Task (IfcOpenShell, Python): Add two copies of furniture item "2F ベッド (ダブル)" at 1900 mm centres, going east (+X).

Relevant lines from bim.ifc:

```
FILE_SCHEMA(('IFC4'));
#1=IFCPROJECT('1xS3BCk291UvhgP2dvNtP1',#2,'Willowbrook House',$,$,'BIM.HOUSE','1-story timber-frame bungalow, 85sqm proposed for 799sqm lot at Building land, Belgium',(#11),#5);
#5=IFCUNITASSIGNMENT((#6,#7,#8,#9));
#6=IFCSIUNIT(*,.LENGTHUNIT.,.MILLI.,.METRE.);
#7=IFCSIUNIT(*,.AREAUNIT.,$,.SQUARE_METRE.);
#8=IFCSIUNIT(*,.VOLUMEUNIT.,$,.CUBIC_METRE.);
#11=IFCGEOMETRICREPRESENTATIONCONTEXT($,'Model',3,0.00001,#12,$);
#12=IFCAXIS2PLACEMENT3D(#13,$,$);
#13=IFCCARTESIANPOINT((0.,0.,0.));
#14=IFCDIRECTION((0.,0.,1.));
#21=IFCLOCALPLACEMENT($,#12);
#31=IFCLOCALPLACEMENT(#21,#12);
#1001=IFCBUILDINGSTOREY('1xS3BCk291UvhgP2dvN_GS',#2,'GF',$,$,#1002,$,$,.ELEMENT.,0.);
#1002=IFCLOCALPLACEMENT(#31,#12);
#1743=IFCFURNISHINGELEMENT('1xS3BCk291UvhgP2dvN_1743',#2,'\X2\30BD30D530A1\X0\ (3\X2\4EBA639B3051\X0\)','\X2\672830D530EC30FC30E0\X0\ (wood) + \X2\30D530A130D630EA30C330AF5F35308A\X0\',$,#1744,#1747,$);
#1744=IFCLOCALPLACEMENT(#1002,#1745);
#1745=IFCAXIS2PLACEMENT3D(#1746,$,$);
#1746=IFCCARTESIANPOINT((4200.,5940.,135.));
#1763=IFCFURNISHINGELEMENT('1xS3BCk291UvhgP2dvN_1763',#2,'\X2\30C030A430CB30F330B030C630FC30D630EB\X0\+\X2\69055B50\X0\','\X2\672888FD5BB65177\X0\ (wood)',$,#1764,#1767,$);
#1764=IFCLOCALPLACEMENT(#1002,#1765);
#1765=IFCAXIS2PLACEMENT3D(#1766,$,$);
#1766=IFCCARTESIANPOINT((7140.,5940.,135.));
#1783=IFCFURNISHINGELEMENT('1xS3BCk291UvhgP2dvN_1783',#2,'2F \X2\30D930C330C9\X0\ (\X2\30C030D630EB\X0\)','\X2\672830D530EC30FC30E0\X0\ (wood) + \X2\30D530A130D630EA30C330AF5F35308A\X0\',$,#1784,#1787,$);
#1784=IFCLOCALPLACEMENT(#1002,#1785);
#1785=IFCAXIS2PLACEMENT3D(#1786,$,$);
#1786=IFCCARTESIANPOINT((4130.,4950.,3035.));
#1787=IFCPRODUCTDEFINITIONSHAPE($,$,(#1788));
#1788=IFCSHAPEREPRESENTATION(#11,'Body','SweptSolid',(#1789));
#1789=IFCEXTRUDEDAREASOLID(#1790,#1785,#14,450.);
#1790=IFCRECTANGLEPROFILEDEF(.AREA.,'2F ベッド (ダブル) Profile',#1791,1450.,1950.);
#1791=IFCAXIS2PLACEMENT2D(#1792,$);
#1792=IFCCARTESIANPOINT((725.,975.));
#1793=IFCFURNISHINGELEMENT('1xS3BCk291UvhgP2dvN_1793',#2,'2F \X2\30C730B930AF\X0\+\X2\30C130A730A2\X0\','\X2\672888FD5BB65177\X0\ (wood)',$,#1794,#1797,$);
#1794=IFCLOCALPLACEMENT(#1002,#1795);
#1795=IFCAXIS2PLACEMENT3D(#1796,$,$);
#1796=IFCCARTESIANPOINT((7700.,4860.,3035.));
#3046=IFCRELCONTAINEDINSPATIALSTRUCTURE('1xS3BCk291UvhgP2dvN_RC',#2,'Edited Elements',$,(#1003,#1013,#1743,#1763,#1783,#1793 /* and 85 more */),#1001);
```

```python
import numpy as np
import ifcopenshell
import ifcopenshell.api.geometry
import ifcopenshell.api.root
import ifcopenshell.util.element
import ifcopenshell.util.placement
import ifcopenshell.util.unit

model = ifcopenshell.open("bim.ifc")
unit_scale = ifcopenshell.util.unit.calculate_unit_scale(model)


def reuse_history(source, copy):
    """copy_class also copies each property set's owner history, people and application; keep the originals."""
    for rel in copy.IsDefinedBy:
        if rel.is_a("IfcRelDefinesByProperties") and (history := rel.RelatingPropertyDefinition.OwnerHistory):
            rel.RelatingPropertyDefinition.OwnerHistory = source.OwnerHistory
            ifcopenshell.util.element.remove_deep2(model, history)


source = model.by_id(1783)
base = ifcopenshell.util.placement.get_local_placement(source.ObjectPlacement)
step = np.array([1.0, 0.0, 0.0]) * 1.9 / unit_scale

for i in range(1, 3):
    copy = ifcopenshell.api.root.copy_class(model, product=source)
    copy.Representation = ifcopenshell.util.element.copy_deep(
        model, source.Representation, exclude=["IfcGeometricRepresentationContext", "IfcRepresentationMap"]
    )
    reuse_history(source, copy)
    matrix = base.copy()
    matrix[:3, 3] += i * step
    print("added at", matrix[:3, 3].round(3) + 0.0)
    ifcopenshell.api.geometry.edit_object_placement(model, product=copy, matrix=matrix, is_si=False)

model.write("bim_v2.ifc")
```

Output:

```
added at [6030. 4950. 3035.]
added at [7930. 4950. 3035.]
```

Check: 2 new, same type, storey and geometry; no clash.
